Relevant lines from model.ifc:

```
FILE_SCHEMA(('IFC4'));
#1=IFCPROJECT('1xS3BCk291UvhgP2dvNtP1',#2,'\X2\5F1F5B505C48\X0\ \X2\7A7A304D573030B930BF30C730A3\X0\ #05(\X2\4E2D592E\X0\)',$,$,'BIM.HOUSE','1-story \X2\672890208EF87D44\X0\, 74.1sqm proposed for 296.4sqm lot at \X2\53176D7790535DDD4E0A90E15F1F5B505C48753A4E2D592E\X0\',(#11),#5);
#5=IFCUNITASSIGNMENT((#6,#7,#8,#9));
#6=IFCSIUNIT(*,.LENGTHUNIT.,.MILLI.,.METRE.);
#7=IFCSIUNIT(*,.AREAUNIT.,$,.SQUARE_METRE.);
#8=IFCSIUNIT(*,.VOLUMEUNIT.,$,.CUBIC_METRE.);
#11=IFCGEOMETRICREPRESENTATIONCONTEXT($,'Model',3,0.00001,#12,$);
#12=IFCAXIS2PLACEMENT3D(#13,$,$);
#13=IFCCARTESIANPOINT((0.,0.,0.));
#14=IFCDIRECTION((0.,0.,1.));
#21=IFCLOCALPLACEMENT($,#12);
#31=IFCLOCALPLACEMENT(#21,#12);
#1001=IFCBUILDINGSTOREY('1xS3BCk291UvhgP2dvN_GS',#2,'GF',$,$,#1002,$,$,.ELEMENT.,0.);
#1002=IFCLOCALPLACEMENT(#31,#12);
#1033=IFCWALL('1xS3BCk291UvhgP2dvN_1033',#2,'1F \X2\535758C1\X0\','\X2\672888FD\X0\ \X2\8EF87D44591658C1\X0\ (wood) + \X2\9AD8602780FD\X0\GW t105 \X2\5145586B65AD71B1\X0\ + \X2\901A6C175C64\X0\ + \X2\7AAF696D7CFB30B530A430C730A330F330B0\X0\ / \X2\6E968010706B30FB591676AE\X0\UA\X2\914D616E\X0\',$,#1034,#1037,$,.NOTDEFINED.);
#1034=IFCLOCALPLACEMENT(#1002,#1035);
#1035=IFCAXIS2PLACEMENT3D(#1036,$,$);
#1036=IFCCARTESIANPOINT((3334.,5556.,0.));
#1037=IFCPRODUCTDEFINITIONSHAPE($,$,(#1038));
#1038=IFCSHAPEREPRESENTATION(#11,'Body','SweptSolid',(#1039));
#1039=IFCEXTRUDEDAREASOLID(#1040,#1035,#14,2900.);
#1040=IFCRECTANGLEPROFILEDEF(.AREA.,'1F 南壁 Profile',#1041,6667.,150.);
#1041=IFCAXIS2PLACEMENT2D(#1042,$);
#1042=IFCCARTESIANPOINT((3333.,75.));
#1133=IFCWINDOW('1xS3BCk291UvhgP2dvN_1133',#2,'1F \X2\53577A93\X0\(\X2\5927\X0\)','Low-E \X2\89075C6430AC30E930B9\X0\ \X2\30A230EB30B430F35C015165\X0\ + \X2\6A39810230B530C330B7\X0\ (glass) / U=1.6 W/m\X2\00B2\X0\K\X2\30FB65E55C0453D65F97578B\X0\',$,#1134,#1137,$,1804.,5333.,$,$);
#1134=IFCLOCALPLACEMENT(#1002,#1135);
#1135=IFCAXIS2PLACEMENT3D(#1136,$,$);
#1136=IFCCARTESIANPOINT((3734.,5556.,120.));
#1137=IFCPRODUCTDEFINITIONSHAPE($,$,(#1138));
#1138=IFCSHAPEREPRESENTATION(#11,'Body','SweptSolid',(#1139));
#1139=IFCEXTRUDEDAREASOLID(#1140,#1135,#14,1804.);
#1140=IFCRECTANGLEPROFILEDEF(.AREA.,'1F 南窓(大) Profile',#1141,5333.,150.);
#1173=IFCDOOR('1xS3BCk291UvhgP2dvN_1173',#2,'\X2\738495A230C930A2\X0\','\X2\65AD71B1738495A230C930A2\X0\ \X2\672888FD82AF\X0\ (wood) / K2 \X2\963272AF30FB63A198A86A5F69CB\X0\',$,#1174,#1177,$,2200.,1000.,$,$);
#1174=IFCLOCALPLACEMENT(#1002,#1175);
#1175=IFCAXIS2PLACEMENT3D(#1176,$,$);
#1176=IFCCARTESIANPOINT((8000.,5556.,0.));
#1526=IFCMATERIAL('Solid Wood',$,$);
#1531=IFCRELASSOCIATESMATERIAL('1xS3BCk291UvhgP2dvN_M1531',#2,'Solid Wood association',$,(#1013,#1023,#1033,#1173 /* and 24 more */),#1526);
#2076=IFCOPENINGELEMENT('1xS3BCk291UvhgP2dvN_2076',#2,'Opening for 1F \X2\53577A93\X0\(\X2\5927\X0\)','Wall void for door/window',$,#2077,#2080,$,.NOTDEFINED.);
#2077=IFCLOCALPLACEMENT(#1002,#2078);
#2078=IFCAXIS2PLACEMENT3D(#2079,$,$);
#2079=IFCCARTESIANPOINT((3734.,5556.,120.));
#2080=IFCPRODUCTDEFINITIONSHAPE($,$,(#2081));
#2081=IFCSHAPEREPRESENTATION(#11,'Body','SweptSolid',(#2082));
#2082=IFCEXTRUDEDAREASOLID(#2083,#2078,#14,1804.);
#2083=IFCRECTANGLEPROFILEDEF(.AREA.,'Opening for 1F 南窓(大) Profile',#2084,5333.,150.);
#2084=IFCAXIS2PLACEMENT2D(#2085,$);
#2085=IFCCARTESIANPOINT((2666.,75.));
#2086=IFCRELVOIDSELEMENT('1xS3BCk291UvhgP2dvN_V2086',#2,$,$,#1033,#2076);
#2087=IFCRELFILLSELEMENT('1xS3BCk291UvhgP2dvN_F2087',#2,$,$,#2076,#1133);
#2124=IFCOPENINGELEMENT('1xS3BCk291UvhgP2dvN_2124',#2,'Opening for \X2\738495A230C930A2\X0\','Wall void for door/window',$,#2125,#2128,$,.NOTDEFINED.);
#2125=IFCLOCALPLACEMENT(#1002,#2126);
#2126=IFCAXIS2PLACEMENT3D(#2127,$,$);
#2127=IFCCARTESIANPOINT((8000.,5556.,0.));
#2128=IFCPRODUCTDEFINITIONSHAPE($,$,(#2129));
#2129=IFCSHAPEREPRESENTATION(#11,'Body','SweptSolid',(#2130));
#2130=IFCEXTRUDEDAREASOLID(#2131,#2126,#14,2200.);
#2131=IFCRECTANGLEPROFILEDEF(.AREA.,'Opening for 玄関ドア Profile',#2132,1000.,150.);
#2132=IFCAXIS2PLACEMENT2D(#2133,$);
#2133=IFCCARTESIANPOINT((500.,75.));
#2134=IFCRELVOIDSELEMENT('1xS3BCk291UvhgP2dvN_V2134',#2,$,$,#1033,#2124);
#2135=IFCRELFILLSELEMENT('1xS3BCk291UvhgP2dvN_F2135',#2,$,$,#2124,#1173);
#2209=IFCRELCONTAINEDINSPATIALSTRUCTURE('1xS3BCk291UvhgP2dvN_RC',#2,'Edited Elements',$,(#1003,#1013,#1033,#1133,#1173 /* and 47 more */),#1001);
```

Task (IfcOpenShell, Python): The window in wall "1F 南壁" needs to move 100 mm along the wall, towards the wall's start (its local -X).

```python
import ifcopenshell
import ifcopenshell.api.geometry
import ifcopenshell.util.placement

model = ifcopenshell.open("model.ifc")

window = model.by_guid("1xS3BCk291UvhgP2dvN_1133")
opening = window.FillsVoids[0].RelatingOpeningElement
wall = opening.VoidsElements[0].RelatingBuildingElement

wall_matrix = ifcopenshell.util.placement.get_local_placement(wall.ObjectPlacement)
shift = wall_matrix[:3, 0] * -100.0
before = ifcopenshell.util.placement.get_local_placement(window.ObjectPlacement)[:3, 3].copy()

# The window is not placed relative to its opening, so move both.
for product in (opening, window):
    matrix = ifcopenshell.util.placement.get_local_placement(product.ObjectPlacement)
    matrix[:3, 3] += shift
    ifcopenshell.api.geometry.edit_object_placement(model, product=product, matrix=matrix, is_si=False)

after = ifcopenshell.util.placement.get_local_placement(window.ObjectPlacement)[:3, 3]
print("window moved by", (after - before).round(3) + 0.0)

model.write("model-out.ifc")
```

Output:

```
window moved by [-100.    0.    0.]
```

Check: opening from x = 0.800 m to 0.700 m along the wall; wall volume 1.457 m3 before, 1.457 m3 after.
